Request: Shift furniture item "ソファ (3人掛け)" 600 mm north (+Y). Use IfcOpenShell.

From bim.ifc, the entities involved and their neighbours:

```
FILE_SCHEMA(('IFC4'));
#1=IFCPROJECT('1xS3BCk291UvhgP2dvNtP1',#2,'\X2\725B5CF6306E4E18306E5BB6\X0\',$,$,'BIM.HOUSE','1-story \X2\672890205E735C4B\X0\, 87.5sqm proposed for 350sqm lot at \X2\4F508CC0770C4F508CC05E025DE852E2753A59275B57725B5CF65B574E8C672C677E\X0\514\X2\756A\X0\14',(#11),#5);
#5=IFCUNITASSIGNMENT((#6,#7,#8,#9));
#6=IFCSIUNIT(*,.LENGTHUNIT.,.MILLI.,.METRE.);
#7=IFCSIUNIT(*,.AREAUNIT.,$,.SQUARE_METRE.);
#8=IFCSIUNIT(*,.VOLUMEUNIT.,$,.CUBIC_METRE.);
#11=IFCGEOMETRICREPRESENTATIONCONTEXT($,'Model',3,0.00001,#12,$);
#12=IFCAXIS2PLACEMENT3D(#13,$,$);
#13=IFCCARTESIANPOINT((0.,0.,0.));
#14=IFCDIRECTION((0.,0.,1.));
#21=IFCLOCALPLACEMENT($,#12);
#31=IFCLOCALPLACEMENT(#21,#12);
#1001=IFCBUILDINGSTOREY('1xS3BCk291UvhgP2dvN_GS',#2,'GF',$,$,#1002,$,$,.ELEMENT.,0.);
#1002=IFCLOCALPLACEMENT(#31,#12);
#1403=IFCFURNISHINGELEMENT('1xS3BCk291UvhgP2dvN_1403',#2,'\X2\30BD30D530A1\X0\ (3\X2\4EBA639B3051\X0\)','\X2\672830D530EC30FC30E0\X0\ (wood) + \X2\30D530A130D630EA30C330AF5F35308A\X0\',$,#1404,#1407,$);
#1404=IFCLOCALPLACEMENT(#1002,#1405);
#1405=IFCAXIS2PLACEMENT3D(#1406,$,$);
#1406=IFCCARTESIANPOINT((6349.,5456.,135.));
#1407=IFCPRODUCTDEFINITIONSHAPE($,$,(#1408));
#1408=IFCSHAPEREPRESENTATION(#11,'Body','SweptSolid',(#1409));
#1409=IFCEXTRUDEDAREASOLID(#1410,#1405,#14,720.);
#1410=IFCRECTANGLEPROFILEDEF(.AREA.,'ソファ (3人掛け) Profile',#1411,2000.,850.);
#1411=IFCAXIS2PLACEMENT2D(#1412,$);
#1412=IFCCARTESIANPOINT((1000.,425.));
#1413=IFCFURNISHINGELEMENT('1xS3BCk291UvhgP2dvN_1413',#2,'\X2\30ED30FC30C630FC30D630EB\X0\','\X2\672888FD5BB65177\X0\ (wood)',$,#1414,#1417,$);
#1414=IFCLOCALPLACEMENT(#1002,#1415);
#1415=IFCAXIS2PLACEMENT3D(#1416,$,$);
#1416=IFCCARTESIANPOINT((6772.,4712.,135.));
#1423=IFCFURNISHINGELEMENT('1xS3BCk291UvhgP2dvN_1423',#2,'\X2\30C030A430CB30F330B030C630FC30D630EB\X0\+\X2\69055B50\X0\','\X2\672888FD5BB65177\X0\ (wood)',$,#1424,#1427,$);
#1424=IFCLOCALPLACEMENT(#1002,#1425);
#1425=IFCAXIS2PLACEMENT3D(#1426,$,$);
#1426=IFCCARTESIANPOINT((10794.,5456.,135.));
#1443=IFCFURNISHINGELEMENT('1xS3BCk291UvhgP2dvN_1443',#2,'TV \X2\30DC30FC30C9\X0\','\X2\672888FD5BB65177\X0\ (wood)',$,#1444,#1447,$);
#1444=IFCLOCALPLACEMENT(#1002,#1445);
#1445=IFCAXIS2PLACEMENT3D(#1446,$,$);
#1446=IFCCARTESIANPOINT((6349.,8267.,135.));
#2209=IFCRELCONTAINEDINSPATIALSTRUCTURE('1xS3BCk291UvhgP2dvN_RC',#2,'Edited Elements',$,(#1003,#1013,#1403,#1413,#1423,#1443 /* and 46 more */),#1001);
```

```python
import ifcopenshell
import ifcopenshell.api.geometry
import ifcopenshell.util.placement
import ifcopenshell.util.unit

model = ifcopenshell.open("bim.ifc")
unit_scale = ifcopenshell.util.unit.calculate_unit_scale(model)

item = model.by_guid("1xS3BCk291UvhgP2dvN_1403")
matrix = ifcopenshell.util.placement.get_local_placement(item.ObjectPlacement)
matrix[1, 3] += 0.6 / unit_scale
ifcopenshell.api.geometry.edit_object_placement(model, product=item, matrix=matrix, is_si=False)

print(ifcopenshell.util.placement.get_local_placement(item.ObjectPlacement).round(3) + 0.0)

model.write("bim-out.ifc")
```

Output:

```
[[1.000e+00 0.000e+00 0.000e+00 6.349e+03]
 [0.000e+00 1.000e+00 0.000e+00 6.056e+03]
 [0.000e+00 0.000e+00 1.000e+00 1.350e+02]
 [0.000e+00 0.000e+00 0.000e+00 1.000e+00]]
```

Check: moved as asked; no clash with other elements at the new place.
